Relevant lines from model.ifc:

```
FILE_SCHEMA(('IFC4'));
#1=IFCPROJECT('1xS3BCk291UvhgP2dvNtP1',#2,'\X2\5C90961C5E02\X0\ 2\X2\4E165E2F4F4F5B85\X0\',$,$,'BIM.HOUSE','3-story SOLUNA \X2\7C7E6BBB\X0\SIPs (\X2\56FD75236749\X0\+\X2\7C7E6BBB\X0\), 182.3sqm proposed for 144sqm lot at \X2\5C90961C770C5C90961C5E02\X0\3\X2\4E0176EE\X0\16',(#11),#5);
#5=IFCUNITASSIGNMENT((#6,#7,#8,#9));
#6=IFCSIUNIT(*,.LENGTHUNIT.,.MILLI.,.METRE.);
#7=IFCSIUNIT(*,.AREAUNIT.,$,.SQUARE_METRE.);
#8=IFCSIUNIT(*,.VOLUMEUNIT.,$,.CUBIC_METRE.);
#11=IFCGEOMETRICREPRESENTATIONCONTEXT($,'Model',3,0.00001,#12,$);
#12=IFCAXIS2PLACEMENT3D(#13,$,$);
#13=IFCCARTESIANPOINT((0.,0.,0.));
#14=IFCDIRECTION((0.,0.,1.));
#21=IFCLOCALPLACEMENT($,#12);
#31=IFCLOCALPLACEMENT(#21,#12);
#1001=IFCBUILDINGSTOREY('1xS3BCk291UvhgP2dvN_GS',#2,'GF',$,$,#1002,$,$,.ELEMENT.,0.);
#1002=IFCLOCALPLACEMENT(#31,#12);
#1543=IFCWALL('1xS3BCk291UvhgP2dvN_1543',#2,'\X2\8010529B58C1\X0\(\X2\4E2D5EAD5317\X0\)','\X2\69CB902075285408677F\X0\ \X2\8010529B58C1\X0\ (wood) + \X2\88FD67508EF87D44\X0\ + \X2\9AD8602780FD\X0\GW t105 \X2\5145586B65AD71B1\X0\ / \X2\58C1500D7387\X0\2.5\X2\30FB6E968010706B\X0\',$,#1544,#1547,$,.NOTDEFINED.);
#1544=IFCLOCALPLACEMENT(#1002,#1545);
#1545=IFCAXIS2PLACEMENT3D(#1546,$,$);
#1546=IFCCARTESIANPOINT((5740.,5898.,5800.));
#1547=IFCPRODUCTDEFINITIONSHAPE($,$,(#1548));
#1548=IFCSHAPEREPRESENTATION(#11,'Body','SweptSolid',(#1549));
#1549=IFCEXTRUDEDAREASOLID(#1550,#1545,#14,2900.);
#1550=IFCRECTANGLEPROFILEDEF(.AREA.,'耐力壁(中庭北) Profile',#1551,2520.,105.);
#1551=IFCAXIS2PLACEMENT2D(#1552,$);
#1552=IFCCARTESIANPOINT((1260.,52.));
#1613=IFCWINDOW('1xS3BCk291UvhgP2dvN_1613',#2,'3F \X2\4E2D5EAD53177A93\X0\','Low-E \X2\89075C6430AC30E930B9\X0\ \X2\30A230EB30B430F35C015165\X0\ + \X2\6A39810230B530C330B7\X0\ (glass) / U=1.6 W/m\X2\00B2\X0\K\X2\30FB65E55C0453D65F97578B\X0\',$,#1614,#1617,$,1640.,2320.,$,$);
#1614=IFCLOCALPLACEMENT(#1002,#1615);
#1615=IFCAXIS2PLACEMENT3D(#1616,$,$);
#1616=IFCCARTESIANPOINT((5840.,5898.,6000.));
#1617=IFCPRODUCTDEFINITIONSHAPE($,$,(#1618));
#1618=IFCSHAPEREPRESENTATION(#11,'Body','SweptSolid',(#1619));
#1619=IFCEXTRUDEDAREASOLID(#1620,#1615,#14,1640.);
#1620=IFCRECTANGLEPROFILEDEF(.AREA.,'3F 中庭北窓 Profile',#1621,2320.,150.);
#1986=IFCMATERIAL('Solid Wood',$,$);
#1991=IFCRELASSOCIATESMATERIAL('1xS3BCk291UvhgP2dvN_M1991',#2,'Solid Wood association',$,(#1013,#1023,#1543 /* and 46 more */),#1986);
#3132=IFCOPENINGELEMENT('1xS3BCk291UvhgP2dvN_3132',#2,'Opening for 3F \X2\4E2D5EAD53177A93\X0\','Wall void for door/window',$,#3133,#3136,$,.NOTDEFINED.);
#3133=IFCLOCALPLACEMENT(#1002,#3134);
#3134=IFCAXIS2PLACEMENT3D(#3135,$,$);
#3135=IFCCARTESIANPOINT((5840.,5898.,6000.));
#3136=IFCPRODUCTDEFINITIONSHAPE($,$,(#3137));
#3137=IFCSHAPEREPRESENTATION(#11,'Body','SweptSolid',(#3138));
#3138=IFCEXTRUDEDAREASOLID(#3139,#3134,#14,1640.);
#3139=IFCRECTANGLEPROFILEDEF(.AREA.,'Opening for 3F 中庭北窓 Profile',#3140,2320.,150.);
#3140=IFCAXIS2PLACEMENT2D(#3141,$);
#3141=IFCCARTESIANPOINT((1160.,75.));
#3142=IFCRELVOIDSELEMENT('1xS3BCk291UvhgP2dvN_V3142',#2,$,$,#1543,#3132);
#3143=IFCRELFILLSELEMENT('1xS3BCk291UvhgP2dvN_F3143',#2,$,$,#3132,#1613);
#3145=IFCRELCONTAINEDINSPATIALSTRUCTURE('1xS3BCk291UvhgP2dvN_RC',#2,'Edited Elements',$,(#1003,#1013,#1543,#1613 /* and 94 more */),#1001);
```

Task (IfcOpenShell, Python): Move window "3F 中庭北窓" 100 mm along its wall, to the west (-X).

```python
import ifcopenshell
import ifcopenshell.api.geometry
import ifcopenshell.util.placement
import ifcopenshell.util.unit

model = ifcopenshell.open("model.ifc")
unit_scale = ifcopenshell.util.unit.calculate_unit_scale(model)

window = model.by_guid("1xS3BCk291UvhgP2dvN_1613")
opening = window.FillsVoids[0].RelatingOpeningElement
wall = opening.VoidsElements[0].RelatingBuildingElement

wall_matrix = ifcopenshell.util.placement.get_local_placement(wall.ObjectPlacement)
shift = wall_matrix[:3, 0] * -0.1 / unit_scale
before = ifcopenshell.util.placement.get_local_placement(window.ObjectPlacement)[:3, 3].copy()

# The window is not placed relative to its opening, so move both.
for product in (opening, window):
    matrix = ifcopenshell.util.placement.get_local_placement(product.ObjectPlacement)
    matrix[:3, 3] += shift
    ifcopenshell.api.geometry.edit_object_placement(model, product=product, matrix=matrix, is_si=False)

after = ifcopenshell.util.placement.get_local_placement(window.ObjectPlacement)[:3, 3]
print("window moved by", (after - before).round(3) + 0.0)

model.write("model_rev.ifc")
```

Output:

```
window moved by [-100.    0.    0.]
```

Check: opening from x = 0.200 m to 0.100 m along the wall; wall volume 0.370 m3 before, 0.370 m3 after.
